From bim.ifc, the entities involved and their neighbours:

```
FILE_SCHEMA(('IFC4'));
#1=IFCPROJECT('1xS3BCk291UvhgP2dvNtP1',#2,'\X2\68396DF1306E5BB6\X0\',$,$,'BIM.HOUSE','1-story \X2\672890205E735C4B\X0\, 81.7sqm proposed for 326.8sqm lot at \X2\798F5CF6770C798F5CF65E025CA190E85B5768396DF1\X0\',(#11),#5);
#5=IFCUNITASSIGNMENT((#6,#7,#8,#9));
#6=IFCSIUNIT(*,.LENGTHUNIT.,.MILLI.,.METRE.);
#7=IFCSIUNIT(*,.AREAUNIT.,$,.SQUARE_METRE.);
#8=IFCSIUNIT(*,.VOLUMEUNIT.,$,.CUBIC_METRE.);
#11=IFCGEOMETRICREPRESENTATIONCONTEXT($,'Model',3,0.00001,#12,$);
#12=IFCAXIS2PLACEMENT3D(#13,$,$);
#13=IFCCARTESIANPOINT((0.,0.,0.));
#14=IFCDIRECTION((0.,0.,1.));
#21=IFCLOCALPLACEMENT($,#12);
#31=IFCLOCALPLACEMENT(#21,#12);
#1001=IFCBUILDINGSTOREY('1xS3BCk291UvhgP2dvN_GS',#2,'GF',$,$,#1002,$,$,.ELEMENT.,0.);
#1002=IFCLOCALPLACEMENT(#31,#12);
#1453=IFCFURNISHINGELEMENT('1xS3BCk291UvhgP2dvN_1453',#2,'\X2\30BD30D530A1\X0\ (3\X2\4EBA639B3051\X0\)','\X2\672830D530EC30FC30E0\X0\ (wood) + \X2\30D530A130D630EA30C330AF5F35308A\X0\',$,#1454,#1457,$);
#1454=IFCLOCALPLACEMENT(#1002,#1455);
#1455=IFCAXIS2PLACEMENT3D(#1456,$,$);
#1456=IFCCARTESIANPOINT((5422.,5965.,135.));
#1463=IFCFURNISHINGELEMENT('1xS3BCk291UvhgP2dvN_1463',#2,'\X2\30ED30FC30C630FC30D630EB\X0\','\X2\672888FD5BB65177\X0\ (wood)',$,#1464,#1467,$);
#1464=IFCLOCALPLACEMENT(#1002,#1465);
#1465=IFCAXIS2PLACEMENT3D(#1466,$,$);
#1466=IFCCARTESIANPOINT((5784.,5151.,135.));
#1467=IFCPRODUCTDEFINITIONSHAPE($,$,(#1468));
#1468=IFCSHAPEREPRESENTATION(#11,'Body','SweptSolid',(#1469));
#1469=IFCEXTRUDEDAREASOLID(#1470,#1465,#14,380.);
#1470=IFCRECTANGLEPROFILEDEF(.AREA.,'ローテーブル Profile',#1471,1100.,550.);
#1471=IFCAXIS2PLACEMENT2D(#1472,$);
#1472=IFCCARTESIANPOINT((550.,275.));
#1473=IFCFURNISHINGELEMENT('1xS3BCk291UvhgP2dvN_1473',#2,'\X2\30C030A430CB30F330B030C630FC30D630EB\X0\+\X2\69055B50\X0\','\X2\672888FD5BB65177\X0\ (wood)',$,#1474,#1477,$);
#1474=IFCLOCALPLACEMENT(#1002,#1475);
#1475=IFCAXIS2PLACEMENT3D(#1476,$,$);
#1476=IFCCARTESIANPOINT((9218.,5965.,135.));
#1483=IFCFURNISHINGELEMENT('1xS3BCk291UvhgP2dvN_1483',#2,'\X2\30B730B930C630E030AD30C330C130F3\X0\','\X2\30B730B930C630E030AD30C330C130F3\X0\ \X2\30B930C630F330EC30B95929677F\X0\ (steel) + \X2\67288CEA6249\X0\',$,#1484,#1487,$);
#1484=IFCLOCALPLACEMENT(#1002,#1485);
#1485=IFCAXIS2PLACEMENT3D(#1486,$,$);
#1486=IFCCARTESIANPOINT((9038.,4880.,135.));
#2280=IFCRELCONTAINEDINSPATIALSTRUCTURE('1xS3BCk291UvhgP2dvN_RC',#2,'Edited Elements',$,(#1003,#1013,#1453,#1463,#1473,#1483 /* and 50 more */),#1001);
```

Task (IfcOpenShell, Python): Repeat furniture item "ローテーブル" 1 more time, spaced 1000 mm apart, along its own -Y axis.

```python
import ifcopenshell
import ifcopenshell.api.geometry
import ifcopenshell.api.root
import ifcopenshell.util.element
import ifcopenshell.util.placement
import ifcopenshell.util.unit

model = ifcopenshell.open("bim.ifc")
unit_scale = ifcopenshell.util.unit.calculate_unit_scale(model)


def reuse_history(source, copy):
    """copy_class also copies each property set's owner history, people and application; keep the originals."""
    for rel in copy.IsDefinedBy:
        if rel.is_a("IfcRelDefinesByProperties") and (history := rel.RelatingPropertyDefinition.OwnerHistory):
            rel.RelatingPropertyDefinition.OwnerHistory = source.OwnerHistory
            ifcopenshell.util.element.remove_deep2(model, history)


source = model.by_guid("1xS3BCk291UvhgP2dvN_1463")
base = ifcopenshell.util.placement.get_local_placement(source.ObjectPlacement)
step = -base[:3, 1] * 1 / unit_scale

for i in range(1, 2):
    copy = ifcopenshell.api.root.copy_class(model, product=source)
    copy.Representation = ifcopenshell.util.element.copy_deep(
        model, source.Representation, exclude=["IfcGeometricRepresentationContext", "IfcRepresentationMap"]
    )
    reuse_history(source, copy)
    matrix = base.copy()
    matrix[:3, 3] += i * step
    print("added at", matrix[:3, 3].round(3) + 0.0)
    ifcopenshell.api.geometry.edit_object_placement(model, product=copy, matrix=matrix, is_si=False)

model.write("bim-out.ifc")
```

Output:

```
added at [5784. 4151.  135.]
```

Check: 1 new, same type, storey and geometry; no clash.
